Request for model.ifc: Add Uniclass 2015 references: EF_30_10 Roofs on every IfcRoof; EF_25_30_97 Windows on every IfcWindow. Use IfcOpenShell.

First a look at what the model holds.

```python
import ifcopenshell

model = ifcopenshell.open("model.ifc")
print(model.schema)
print("classifications:", [c.Name for c in model.by_type("IfcClassification")])
for ifc_class in ("IfcDoor", "IfcRoof", "IfcStair", "IfcWall", "IfcWindow"):
    print(ifc_class, len(model.by_type(ifc_class)))
```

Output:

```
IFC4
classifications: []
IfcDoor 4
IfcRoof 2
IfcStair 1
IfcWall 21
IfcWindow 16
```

```python
import ifcopenshell
import ifcopenshell.api.classification

model = ifcopenshell.open("model.ifc")

system = ifcopenshell.api.classification.add_classification(model, classification="Uniclass 2015")

codes = {
    "IfcRoof": ("EF_30_10", "Roofs"),
    "IfcWindow": ("EF_25_30_97", "Windows"),
}
for ifc_class, (code, name) in codes.items():
    products = model.by_type(ifc_class)
    ifcopenshell.api.classification.add_reference(
        model, products=products, classification=system, identification=code, name=name
    )
    print(code, len(products))

model.write("model_edited.ifc")
```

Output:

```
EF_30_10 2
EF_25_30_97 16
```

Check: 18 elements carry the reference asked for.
